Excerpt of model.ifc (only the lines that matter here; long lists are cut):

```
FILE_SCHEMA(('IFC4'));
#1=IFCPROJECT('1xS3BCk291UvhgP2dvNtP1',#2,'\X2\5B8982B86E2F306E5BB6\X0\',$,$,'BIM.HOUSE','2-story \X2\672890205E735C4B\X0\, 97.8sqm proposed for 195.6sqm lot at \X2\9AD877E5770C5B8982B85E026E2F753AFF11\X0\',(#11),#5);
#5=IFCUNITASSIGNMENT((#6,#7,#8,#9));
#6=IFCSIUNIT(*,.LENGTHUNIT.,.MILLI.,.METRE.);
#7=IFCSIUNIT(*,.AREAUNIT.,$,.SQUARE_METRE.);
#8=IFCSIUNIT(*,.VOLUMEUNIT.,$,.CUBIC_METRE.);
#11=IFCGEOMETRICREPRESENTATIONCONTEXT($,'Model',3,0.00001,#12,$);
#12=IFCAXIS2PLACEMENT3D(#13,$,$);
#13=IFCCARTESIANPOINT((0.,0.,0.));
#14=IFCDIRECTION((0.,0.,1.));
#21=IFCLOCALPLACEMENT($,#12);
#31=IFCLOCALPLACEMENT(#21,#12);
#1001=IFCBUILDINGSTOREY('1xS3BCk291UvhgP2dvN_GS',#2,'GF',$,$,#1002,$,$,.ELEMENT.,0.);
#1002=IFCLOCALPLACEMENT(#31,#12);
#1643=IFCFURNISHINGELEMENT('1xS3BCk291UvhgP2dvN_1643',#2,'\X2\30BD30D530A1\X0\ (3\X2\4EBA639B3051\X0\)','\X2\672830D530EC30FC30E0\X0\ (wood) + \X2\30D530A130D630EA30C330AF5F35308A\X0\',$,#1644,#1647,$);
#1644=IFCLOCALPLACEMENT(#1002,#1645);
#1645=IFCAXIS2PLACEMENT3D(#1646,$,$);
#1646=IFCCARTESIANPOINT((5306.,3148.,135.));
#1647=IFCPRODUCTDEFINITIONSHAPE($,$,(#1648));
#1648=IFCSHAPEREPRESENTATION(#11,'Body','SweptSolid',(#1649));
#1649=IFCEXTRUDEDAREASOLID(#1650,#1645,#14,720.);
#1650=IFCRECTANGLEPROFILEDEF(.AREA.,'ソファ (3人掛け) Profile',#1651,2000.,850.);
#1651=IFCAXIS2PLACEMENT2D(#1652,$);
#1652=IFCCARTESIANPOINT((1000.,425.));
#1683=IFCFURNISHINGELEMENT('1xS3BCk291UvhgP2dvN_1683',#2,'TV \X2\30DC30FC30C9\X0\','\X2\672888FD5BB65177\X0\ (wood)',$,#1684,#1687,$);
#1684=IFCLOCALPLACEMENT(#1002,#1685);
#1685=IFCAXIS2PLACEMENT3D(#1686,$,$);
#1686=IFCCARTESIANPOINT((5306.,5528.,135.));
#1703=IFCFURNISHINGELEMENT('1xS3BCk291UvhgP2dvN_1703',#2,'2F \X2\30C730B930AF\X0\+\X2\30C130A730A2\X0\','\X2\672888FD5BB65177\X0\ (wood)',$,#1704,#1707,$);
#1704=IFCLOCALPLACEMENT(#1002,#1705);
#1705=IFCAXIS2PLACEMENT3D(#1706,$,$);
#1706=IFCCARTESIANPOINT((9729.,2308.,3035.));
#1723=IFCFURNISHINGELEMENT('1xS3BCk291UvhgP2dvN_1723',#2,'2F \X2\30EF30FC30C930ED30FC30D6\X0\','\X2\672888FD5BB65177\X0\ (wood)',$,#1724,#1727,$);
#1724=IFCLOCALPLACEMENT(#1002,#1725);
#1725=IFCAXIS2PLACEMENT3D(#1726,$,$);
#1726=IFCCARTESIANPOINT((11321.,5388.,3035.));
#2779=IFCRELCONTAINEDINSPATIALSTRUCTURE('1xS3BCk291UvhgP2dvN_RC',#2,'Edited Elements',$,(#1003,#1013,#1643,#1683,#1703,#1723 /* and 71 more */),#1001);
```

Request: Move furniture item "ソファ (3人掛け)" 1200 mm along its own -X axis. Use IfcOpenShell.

```python
import ifcopenshell
import ifcopenshell.api.geometry
import ifcopenshell.util.placement
import ifcopenshell.util.unit

model = ifcopenshell.open("model.ifc")
unit_scale = ifcopenshell.util.unit.calculate_unit_scale(model)

item = model.by_guid("1xS3BCk291UvhgP2dvN_1643")
matrix = ifcopenshell.util.placement.get_local_placement(item.ObjectPlacement)
matrix[:3, 3] -= matrix[:3, 0] * 1.2 / unit_scale
ifcopenshell.api.geometry.edit_object_placement(model, product=item, matrix=matrix, is_si=False)

print(ifcopenshell.util.placement.get_local_placement(item.ObjectPlacement).round(3) + 0.0)

model.write("model_rev.ifc")
```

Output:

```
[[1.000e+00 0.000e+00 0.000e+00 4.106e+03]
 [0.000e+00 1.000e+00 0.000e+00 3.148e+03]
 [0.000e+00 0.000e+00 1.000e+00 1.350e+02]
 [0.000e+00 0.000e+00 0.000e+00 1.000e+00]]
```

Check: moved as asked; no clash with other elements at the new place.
